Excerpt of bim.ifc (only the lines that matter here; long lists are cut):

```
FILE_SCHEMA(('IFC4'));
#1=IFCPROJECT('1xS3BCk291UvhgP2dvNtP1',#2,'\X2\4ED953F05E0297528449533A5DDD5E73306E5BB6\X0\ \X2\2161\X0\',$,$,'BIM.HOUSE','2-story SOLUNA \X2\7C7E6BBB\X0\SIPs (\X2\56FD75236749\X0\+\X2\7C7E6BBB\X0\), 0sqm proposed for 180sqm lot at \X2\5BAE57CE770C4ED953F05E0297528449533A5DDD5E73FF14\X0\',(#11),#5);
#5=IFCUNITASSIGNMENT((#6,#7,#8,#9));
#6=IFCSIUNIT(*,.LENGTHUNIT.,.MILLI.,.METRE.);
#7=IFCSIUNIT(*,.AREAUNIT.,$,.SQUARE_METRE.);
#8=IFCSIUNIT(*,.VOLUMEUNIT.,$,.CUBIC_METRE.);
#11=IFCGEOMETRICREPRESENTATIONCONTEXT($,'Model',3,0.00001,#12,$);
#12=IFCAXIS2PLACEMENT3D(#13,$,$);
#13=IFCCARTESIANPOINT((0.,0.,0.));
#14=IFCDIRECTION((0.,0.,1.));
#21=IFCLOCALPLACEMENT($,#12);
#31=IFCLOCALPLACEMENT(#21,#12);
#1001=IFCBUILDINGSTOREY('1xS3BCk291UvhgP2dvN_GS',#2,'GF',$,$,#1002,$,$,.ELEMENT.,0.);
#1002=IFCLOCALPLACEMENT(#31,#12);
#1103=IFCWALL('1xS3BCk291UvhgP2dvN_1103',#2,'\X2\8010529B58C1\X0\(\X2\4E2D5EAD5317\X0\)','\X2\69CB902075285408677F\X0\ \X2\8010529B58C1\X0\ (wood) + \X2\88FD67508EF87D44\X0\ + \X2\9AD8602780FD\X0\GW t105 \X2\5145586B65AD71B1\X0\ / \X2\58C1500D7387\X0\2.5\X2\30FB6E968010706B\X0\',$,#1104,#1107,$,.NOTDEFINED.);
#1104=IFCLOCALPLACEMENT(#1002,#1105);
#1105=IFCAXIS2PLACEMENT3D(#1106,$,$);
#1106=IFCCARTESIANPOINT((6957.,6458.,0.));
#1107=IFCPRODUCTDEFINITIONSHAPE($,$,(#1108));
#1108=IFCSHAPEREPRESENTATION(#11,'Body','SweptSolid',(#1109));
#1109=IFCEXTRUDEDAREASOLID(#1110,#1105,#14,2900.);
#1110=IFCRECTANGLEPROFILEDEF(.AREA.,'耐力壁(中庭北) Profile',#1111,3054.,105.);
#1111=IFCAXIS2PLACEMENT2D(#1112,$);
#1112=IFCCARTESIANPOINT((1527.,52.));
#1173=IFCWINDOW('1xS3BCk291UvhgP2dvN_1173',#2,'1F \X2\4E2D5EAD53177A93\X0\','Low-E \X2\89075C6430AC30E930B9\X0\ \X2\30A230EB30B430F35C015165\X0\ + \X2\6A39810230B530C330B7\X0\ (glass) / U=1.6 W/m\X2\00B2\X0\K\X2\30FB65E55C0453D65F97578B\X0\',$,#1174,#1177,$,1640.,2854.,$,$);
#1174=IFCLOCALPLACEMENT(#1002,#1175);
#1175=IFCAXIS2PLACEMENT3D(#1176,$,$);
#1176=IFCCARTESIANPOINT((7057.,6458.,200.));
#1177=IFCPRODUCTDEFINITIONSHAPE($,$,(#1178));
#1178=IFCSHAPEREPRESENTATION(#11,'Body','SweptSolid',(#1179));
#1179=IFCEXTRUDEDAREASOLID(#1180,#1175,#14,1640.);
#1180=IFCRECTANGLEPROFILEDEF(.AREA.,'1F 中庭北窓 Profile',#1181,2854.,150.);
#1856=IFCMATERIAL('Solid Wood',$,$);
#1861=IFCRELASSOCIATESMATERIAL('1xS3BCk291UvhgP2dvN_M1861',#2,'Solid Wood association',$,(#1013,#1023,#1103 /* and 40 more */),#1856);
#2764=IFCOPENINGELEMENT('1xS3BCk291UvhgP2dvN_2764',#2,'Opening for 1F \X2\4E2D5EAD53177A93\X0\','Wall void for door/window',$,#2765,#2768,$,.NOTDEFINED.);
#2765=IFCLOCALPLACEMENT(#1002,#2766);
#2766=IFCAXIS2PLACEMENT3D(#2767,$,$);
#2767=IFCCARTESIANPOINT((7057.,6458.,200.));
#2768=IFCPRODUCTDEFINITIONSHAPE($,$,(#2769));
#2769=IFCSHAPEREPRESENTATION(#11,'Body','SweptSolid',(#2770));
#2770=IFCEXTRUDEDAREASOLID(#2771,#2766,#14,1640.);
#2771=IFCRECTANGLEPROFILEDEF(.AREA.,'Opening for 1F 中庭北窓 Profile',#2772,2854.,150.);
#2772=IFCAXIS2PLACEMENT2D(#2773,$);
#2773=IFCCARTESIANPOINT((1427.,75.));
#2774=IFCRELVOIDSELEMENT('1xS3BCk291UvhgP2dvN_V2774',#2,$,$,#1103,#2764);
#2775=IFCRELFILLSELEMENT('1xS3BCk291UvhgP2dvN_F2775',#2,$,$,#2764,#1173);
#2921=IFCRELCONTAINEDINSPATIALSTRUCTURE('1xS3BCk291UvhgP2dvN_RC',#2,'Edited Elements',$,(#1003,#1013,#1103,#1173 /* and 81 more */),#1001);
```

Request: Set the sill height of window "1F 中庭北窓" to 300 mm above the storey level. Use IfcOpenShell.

```python
import numpy as np
import ifcopenshell
import ifcopenshell.api.geometry
import ifcopenshell.geom
import ifcopenshell.util.element
import ifcopenshell.util.placement
import ifcopenshell.util.shape
import ifcopenshell.util.unit

model = ifcopenshell.open("bim.ifc")
unit_scale = ifcopenshell.util.unit.calculate_unit_scale(model)

window = model.by_guid("1xS3BCk291UvhgP2dvN_1173")
opening = window.FillsVoids[0].RelatingOpeningElement
storey = ifcopenshell.util.element.get_container(window, ifc_class="IfcBuildingStorey")
level = ifcopenshell.util.placement.get_local_placement(storey.ObjectPlacement)[2, 3]

# The opening's origin need not be at the sill, so measure its lowest point.
shape = ifcopenshell.geom.create_shape(ifcopenshell.geom.settings(), opening)
bottom = ifcopenshell.util.shape.get_shape_bottom_elevation(shape, shape.geometry) / unit_scale
dz = level + 300.0 - bottom

shift = np.array([0.0, 0.0, dz])
# The window is not placed relative to its opening, so move both.
for product in (opening, window):
    matrix = ifcopenshell.util.placement.get_local_placement(product.ObjectPlacement)
    matrix[:3, 3] += shift
    ifcopenshell.api.geometry.edit_object_placement(model, product=product, matrix=matrix, is_si=False)

print(f"moved by {dz * unit_scale:+.3f} m")

model.write("bim_v2.ifc")
```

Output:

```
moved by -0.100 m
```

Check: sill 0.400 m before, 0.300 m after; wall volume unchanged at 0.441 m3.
